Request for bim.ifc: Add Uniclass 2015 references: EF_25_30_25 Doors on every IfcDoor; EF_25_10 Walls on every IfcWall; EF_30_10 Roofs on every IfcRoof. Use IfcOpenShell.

First a look at what the model holds.

```python
import ifcopenshell

model = ifcopenshell.open("bim.ifc")
print(model.schema)
print("classifications:", [c.Name for c in model.by_type("IfcClassification")])
for ifc_class in ("IfcDoor", "IfcRoof", "IfcStair", "IfcWall", "IfcWindow"):
    print(ifc_class, len(model.by_type(ifc_class)))
```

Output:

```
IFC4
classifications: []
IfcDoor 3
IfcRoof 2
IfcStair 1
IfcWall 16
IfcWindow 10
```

```python
import ifcopenshell
import ifcopenshell.api.classification

model = ifcopenshell.open("bim.ifc")

system = ifcopenshell.api.classification.add_classification(model, classification="Uniclass 2015")

codes = {
    "IfcDoor": ("EF_25_30_25", "Doors"),
    "IfcWall": ("EF_25_10", "Walls"),
    "IfcRoof": ("EF_30_10", "Roofs"),
}
for ifc_class, (code, name) in codes.items():
    products = model.by_type(ifc_class)
    ifcopenshell.api.classification.add_reference(
        model, products=products, classification=system, identification=code, name=name
    )
    print(code, len(products))

model.write("bim_v2.ifc")
```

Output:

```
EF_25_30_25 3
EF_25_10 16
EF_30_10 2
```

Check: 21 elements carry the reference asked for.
